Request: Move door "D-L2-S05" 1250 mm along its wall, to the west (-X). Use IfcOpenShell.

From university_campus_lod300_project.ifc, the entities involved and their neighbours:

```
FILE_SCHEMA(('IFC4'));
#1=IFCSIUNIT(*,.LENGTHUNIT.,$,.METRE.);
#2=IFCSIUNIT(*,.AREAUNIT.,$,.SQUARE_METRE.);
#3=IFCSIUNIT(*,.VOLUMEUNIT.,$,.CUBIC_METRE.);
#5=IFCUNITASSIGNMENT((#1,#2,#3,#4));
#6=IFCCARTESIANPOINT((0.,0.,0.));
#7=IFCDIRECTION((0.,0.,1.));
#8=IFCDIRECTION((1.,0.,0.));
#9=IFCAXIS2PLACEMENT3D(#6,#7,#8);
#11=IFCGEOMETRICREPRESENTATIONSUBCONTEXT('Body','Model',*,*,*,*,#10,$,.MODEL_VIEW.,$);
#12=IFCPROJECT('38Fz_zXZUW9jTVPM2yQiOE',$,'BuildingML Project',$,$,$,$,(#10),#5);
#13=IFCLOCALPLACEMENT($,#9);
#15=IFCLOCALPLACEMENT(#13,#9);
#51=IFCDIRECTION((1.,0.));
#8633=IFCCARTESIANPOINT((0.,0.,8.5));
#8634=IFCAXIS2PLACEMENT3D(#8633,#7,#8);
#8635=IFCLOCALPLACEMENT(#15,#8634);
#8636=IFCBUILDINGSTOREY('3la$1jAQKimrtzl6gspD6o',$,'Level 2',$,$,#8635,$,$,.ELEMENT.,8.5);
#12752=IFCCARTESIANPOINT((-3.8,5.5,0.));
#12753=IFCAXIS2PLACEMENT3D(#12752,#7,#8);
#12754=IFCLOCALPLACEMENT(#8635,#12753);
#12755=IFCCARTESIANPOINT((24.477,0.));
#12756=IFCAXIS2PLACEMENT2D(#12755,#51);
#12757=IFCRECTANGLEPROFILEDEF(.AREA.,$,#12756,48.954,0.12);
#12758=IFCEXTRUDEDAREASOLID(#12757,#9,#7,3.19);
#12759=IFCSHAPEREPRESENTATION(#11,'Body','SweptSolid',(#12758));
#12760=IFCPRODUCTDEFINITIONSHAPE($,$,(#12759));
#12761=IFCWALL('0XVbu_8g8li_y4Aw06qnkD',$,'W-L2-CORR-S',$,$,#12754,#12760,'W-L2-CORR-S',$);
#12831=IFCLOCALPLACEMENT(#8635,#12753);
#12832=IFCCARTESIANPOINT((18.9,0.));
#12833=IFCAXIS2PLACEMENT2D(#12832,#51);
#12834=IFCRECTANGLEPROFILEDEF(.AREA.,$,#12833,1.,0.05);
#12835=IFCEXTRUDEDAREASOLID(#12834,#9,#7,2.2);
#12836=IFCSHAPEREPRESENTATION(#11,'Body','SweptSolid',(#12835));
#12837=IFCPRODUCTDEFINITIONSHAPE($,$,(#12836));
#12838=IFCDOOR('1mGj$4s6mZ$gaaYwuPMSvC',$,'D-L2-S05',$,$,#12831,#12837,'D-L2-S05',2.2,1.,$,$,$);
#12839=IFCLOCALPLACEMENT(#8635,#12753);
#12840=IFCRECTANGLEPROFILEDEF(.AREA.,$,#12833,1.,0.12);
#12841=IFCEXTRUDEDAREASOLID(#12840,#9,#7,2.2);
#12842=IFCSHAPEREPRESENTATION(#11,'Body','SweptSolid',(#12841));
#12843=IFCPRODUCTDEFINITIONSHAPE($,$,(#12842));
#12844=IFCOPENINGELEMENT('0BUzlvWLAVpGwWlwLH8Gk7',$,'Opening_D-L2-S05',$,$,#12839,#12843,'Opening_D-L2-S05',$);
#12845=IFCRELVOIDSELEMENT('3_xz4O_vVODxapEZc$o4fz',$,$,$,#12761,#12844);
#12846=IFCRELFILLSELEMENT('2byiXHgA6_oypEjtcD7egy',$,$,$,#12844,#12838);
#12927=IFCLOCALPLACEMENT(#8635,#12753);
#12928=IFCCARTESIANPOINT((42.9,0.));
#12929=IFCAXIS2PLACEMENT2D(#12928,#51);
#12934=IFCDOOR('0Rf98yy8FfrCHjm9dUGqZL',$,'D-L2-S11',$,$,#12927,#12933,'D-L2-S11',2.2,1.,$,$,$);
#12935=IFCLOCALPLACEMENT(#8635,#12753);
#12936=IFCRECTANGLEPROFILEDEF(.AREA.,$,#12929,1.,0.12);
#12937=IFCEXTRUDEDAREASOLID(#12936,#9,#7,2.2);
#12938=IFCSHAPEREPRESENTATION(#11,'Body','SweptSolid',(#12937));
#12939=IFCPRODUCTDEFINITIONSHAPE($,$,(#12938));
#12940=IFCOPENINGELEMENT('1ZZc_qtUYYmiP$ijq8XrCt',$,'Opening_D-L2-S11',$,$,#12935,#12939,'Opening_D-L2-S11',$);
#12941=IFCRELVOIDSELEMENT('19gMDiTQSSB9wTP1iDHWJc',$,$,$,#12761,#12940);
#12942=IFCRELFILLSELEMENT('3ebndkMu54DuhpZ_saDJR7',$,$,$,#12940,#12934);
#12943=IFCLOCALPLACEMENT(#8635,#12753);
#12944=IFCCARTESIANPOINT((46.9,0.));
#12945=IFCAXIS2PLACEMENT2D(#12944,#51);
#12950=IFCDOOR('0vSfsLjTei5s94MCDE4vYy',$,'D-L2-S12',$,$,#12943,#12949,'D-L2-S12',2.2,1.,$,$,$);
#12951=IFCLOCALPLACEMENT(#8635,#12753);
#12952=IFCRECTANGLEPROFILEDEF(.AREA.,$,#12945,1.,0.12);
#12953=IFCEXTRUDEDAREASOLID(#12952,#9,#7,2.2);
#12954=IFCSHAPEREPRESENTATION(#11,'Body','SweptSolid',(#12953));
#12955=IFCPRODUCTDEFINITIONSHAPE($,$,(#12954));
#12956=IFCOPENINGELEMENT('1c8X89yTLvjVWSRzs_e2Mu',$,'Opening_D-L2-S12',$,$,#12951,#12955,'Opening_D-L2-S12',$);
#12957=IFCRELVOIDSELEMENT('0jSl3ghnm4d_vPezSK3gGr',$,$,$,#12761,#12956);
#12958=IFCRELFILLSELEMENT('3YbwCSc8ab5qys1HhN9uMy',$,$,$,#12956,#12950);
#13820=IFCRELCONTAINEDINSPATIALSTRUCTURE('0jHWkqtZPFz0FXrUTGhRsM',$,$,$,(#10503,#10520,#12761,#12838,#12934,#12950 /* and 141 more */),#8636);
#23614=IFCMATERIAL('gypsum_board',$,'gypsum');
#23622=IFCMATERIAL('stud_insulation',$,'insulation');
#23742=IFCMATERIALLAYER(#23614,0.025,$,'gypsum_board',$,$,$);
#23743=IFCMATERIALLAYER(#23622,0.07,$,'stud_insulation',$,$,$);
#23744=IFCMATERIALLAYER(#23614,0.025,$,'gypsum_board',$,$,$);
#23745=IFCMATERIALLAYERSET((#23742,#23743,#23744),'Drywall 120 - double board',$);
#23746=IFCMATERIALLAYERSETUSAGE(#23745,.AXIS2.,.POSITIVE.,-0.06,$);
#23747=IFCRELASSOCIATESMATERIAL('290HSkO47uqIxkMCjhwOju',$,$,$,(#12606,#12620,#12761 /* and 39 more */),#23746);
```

```python
import ifcopenshell
import ifcopenshell.api.geometry
import ifcopenshell.util.placement
import ifcopenshell.util.unit

model = ifcopenshell.open("university_campus_lod300_project.ifc")
unit_scale = ifcopenshell.util.unit.calculate_unit_scale(model)

door = model.by_guid("1mGj$4s6mZ$gaaYwuPMSvC")
opening = door.FillsVoids[0].RelatingOpeningElement
wall = opening.VoidsElements[0].RelatingBuildingElement

wall_matrix = ifcopenshell.util.placement.get_local_placement(wall.ObjectPlacement)
shift = wall_matrix[:3, 0] * -1.25 / unit_scale
before = ifcopenshell.util.placement.get_local_placement(door.ObjectPlacement)[:3, 3].copy()

# The door is not placed relative to its opening, so move both.
for product in (opening, door):
    matrix = ifcopenshell.util.placement.get_local_placement(product.ObjectPlacement)
    matrix[:3, 3] += shift
    ifcopenshell.api.geometry.edit_object_placement(model, product=product, matrix=matrix, is_si=False)

after = ifcopenshell.util.placement.get_local_placement(door.ObjectPlacement)[:3, 3]
print("door moved by", (after - before).round(3) + 0.0)

model.write("university_campus_lod300_project_rev.ifc")
```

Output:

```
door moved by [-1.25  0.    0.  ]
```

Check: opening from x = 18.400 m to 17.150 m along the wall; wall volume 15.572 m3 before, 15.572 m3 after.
